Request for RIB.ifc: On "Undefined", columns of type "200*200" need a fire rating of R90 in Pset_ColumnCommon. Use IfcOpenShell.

First a look at what the model holds.

```python
import ifcopenshell
import ifcopenshell.util.element

model = ifcopenshell.open("RIB.ifc")
print(model.schema)
storey = next(s for s in model.by_type("IfcBuildingStorey") if s.Name == "Undefined")
columns = [e for e in ifcopenshell.util.element.get_decomposition(storey) if e.is_a("IfcColumn")]
seen = {}
for e in columns:
    element_type = ifcopenshell.util.element.get_type(e)
    key = (element_type.Name if element_type != e and element_type else None, ifcopenshell.util.element.get_pset(e, "Pset_ColumnCommon", "FireRating"))
    seen[key] = seen.get(key, 0) + 1
for (name, value), count in sorted(seen.items(), key=str):
    print(count, "x", name, "|", value)
```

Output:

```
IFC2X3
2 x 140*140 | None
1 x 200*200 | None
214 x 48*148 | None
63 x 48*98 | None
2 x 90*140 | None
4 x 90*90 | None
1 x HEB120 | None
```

```python
import ifcopenshell
import ifcopenshell.api.pset
import ifcopenshell.util.element

model = ifcopenshell.open("RIB.ifc")

storey = next(s for s in model.by_type("IfcBuildingStorey") if s.Name == "Undefined")
columns = [e for e in ifcopenshell.util.element.get_decomposition(storey) if e.is_a("IfcColumn")]

count = 0
for e in columns:
    element_type = ifcopenshell.util.element.get_type(e)
    if element_type in (None, e) or element_type.Name != "200*200":
        continue
    # add_pset returns the element's existing set when there is one.
    pset = ifcopenshell.api.pset.add_pset(model, product=e, name="Pset_ColumnCommon")
    ifcopenshell.api.pset.edit_pset(model, pset=pset, properties={"FireRating": "R90"})
    count += 1

print(count, "columns updated")

model.write("RIB-out.ifc")
```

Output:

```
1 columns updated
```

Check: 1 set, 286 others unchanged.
